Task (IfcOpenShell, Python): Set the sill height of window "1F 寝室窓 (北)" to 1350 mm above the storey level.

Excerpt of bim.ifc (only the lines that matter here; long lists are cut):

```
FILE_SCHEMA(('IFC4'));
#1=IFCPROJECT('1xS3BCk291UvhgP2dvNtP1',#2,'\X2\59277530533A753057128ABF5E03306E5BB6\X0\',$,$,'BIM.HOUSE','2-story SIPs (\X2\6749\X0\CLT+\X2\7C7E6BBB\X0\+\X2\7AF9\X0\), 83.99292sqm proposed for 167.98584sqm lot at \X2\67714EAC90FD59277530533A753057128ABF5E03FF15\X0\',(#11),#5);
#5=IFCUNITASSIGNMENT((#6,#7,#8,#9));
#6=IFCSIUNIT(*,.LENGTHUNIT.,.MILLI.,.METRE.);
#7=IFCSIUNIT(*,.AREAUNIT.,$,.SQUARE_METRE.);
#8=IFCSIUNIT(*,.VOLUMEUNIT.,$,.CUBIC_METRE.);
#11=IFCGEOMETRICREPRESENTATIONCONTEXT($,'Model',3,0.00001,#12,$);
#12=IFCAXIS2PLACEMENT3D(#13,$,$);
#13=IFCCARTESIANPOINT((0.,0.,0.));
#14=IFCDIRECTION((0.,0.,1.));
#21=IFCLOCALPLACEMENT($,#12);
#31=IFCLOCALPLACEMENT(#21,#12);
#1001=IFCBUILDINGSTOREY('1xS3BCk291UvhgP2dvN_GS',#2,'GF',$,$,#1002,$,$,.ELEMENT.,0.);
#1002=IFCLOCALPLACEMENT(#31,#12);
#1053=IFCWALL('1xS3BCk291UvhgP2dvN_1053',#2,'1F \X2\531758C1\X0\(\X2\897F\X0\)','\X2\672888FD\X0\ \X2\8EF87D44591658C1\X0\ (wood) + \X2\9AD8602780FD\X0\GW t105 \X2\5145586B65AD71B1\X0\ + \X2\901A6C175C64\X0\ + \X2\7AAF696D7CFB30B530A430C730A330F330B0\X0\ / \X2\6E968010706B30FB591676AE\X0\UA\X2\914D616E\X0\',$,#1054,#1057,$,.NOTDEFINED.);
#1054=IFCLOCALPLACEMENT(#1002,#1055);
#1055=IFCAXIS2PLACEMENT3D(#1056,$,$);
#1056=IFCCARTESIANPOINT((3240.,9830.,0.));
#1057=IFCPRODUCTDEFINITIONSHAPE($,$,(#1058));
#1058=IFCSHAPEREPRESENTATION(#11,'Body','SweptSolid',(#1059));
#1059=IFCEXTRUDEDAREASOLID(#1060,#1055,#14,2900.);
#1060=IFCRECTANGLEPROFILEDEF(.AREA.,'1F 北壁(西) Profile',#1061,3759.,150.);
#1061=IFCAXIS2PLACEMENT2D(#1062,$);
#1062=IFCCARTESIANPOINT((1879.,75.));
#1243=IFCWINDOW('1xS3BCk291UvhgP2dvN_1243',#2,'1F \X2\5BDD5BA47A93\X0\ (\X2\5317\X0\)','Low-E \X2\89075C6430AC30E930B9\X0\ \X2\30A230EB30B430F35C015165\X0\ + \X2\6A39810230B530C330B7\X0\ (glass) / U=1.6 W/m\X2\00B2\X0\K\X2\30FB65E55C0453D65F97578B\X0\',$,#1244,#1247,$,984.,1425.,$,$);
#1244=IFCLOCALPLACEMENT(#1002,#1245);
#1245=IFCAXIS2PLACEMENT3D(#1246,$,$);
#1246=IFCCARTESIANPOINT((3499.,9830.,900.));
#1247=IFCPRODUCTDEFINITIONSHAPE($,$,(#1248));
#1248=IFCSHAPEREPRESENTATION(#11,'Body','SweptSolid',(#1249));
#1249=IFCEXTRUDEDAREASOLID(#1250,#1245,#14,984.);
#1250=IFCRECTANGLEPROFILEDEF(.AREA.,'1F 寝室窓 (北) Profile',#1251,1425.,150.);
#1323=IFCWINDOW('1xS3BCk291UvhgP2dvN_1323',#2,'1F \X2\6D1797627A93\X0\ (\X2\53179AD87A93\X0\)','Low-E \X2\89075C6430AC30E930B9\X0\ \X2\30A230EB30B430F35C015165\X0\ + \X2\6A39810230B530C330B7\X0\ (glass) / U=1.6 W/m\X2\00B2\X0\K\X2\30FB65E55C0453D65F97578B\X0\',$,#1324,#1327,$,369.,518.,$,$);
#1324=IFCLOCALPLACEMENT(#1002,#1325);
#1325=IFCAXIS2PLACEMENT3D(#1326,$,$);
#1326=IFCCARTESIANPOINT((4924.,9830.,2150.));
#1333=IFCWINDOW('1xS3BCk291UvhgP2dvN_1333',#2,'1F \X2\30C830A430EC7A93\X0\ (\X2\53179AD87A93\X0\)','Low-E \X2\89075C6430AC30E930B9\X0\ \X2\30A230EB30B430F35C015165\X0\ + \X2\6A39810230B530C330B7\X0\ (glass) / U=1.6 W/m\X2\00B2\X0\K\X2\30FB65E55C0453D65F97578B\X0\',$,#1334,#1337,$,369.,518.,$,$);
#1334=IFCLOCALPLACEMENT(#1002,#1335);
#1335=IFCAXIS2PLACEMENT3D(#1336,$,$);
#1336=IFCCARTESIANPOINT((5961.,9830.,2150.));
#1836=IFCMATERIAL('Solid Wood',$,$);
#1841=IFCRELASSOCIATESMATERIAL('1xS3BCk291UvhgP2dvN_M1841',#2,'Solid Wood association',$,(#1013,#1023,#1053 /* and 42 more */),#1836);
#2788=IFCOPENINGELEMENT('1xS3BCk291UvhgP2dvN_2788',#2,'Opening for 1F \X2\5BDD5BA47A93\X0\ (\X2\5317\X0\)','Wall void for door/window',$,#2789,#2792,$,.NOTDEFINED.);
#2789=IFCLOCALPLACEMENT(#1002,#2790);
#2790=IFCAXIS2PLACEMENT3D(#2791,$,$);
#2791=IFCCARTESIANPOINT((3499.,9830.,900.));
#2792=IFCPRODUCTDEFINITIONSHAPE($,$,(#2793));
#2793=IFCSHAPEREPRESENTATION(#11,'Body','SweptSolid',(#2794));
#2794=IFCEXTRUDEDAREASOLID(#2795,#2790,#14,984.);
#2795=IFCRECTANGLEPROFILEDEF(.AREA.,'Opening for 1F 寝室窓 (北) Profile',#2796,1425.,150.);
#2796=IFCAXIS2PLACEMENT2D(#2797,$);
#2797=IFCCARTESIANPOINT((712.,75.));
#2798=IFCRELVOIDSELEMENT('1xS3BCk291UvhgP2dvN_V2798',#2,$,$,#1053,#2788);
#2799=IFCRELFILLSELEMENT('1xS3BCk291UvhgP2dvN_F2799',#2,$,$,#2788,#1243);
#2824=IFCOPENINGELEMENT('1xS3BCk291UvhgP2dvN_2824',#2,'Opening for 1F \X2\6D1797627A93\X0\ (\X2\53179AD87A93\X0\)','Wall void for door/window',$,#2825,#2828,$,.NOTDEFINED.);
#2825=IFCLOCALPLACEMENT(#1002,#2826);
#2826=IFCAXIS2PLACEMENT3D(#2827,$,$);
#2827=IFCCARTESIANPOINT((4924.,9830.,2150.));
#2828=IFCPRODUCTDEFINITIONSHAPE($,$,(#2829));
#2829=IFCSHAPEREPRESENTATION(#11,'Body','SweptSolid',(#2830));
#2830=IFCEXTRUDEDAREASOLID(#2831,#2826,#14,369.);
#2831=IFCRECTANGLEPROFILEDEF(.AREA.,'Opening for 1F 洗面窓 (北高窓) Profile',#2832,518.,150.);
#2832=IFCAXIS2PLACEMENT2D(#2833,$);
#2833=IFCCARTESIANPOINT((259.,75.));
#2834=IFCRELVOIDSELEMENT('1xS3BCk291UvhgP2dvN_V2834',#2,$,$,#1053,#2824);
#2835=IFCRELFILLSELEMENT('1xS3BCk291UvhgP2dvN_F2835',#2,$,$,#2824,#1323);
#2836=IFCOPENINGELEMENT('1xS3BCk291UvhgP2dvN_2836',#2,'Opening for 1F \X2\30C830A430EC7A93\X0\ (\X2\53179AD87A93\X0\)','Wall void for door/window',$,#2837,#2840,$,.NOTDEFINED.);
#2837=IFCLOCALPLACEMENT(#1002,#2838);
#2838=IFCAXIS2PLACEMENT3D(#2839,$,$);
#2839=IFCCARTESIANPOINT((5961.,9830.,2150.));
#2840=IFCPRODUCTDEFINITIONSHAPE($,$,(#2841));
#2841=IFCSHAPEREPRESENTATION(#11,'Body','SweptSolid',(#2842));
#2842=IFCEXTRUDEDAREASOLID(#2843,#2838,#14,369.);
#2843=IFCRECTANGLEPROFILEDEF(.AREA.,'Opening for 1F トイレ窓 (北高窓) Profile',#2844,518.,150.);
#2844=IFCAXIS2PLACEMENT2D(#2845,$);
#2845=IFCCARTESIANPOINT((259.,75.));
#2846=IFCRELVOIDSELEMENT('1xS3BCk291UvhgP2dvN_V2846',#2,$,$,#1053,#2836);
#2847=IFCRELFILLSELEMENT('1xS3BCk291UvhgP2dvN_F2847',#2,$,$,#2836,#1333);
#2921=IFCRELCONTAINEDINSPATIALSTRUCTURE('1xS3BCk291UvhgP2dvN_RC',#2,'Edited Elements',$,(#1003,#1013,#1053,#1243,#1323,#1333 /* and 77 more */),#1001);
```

```python
import numpy as np
import ifcopenshell
import ifcopenshell.api.geometry
import ifcopenshell.geom
import ifcopenshell.util.element
import ifcopenshell.util.placement
import ifcopenshell.util.shape
import ifcopenshell.util.unit

model = ifcopenshell.open("bim.ifc")
unit_scale = ifcopenshell.util.unit.calculate_unit_scale(model)

window = model.by_id(1243)
opening = window.FillsVoids[0].RelatingOpeningElement
storey = ifcopenshell.util.element.get_container(window, ifc_class="IfcBuildingStorey")
level = ifcopenshell.util.placement.get_local_placement(storey.ObjectPlacement)[2, 3]

# The opening's origin need not be at the sill, so measure its lowest point.
shape = ifcopenshell.geom.create_shape(ifcopenshell.geom.settings(), opening)
bottom = ifcopenshell.util.shape.get_shape_bottom_elevation(shape, shape.geometry) / unit_scale
dz = level + 1.35 / unit_scale - bottom

shift = np.array([0.0, 0.0, dz])
# The window is not placed relative to its opening, so move both.
for product in (opening, window):
    matrix = ifcopenshell.util.placement.get_local_placement(product.ObjectPlacement)
    matrix[:3, 3] += shift
    ifcopenshell.api.geometry.edit_object_placement(model, product=product, matrix=matrix, is_si=False)

print(f"moved by {dz * unit_scale:+.3f} m")

model.write("bim_v2.ifc")
```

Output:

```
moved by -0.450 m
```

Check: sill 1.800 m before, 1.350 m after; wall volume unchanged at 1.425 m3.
